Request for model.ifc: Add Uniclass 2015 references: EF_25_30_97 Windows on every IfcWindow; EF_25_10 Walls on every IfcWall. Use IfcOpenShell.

First a look at what the model holds.

```python
import ifcopenshell

model = ifcopenshell.open("model.ifc")
print(model.schema)
print("classifications:", [c.Name for c in model.by_type("IfcClassification")])
for ifc_class in ("IfcDoor", "IfcRoof", "IfcStair", "IfcWall", "IfcWindow"):
    print(ifc_class, len(model.by_type(ifc_class)))
```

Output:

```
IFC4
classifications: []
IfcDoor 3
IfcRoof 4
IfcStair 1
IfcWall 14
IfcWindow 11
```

```python
import ifcopenshell
import ifcopenshell.api.classification

model = ifcopenshell.open("model.ifc")

system = ifcopenshell.api.classification.add_classification(model, classification="Uniclass 2015")

codes = {
    "IfcWindow": ("EF_25_30_97", "Windows"),
    "IfcWall": ("EF_25_10", "Walls"),
}
for ifc_class, (code, name) in codes.items():
    products = model.by_type(ifc_class)
    ifcopenshell.api.classification.add_reference(
        model, products=products, classification=system, identification=code, name=name
    )
    print(code, len(products))

model.write("model-out.ifc")
```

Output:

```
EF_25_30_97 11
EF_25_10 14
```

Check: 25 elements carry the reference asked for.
